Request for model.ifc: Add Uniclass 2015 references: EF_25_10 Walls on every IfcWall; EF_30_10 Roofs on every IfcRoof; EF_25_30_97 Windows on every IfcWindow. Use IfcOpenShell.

First a look at what the model holds.

```python
import ifcopenshell

model = ifcopenshell.open("model.ifc")
print(model.schema)
print("classifications:", [c.Name for c in model.by_type("IfcClassification")])
for ifc_class in ("IfcDoor", "IfcRoof", "IfcStair", "IfcWall", "IfcWindow"):
    print(ifc_class, len(model.by_type(ifc_class)))
```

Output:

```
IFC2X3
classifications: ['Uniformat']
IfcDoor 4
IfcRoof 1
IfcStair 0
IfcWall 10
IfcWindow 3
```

```python
import ifcopenshell
import ifcopenshell.api.classification

model = ifcopenshell.open("model.ifc")

# IFC2X3 requires Source and Edition and has no link from the project to the system.
system = model.create_entity("IfcClassification", Source="NBS", Edition="2015", Name="Uniclass 2015")

codes = {
    "IfcWall": ("EF_25_10", "Walls"),
    "IfcRoof": ("EF_30_10", "Roofs"),
    "IfcWindow": ("EF_25_30_97", "Windows"),
}
for ifc_class, (code, name) in codes.items():
    products = model.by_type(ifc_class)
    ifcopenshell.api.classification.add_reference(
        model, products=products, classification=system, identification=code, name=name
    )
    print(code, len(products))

model.write("model_edited.ifc")
```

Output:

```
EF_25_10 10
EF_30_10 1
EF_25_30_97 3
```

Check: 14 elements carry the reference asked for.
